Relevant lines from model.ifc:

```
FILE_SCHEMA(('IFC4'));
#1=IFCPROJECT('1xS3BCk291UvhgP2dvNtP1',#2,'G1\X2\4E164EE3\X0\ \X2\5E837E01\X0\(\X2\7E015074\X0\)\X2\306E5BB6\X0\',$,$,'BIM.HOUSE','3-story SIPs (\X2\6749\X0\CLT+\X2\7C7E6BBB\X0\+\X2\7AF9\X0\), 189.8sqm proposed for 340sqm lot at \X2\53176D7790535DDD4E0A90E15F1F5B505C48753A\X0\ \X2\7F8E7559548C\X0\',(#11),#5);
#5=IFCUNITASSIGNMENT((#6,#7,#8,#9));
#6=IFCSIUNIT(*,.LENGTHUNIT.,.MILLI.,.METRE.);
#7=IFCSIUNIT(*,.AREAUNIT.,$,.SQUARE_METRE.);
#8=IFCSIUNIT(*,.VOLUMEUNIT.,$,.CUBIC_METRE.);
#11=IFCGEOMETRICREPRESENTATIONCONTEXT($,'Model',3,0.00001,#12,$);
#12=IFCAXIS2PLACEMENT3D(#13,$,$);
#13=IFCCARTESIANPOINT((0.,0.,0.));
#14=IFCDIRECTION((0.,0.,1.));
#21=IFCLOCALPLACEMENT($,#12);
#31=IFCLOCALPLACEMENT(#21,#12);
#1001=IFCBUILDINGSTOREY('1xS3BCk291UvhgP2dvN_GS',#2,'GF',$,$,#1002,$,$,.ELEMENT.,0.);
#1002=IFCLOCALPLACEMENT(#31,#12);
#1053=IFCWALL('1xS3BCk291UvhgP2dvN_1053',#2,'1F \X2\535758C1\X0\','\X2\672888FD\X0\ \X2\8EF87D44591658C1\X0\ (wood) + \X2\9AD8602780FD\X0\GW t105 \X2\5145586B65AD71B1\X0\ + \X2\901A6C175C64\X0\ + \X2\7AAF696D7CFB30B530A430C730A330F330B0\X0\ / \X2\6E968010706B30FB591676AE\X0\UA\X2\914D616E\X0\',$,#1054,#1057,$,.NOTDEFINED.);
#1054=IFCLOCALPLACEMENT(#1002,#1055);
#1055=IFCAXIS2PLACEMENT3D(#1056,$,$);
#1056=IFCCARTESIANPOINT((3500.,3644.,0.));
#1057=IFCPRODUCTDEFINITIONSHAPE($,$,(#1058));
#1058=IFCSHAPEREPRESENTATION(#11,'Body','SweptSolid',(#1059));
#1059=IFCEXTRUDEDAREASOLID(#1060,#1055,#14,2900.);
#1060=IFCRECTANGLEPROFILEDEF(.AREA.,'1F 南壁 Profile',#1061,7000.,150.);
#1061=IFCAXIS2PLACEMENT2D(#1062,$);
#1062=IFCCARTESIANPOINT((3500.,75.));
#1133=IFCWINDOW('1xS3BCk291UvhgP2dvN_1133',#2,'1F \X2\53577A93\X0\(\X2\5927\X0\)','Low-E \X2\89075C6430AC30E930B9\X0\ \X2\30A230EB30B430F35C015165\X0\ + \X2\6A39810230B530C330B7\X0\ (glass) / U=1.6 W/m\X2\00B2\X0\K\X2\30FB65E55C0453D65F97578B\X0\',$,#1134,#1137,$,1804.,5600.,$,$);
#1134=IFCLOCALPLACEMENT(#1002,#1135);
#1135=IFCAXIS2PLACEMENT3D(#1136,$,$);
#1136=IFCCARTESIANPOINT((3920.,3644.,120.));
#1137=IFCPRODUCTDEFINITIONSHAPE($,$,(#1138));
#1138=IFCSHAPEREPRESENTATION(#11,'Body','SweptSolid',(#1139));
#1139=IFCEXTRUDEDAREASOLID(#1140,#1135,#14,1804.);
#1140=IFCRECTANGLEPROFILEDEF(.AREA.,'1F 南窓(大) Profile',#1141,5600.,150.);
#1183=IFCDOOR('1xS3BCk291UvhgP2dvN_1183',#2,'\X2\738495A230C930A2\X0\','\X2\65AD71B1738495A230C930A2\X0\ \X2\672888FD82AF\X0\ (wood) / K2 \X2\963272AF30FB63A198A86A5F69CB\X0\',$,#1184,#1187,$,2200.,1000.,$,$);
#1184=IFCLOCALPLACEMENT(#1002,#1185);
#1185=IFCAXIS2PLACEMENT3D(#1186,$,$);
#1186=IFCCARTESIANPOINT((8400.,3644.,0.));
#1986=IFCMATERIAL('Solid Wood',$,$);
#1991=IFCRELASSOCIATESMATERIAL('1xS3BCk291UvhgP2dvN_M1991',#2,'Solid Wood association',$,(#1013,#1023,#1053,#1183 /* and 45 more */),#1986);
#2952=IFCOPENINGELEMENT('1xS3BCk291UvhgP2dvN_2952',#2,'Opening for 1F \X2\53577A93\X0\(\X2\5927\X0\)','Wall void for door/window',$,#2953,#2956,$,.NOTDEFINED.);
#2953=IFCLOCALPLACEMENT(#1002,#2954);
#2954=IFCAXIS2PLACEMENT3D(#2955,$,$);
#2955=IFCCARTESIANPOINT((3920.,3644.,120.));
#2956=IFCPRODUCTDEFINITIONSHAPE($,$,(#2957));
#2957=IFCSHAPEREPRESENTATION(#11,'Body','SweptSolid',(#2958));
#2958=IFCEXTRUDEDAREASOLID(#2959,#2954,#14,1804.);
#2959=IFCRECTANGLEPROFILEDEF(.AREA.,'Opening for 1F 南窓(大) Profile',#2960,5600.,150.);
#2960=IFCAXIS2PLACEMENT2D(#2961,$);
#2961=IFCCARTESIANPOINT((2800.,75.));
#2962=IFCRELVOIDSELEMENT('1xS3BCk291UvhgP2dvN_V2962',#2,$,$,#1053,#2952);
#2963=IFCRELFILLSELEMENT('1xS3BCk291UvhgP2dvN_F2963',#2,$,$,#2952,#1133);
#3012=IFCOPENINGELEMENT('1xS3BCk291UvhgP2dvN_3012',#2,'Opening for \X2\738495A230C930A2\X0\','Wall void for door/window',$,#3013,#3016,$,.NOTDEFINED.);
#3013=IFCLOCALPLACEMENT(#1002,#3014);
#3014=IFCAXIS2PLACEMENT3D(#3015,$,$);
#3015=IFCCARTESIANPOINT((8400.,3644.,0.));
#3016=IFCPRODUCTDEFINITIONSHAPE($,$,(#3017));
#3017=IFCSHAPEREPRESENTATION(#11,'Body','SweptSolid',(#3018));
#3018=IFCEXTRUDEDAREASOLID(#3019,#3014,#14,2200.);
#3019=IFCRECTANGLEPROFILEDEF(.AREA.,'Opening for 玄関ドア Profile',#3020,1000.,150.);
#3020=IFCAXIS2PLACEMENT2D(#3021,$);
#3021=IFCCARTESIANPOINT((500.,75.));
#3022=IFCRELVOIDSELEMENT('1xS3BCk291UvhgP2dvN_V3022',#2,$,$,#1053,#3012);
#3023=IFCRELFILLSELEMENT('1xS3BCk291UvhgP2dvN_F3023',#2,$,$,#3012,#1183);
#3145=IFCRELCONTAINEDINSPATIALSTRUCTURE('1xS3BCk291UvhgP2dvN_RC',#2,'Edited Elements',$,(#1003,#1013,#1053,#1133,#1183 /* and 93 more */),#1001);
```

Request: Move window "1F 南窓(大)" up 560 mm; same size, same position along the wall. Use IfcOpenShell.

```python
import numpy as np
import ifcopenshell
import ifcopenshell.api.geometry
import ifcopenshell.util.placement
import ifcopenshell.util.unit

model = ifcopenshell.open("model.ifc")
unit_scale = ifcopenshell.util.unit.calculate_unit_scale(model)

window = model.by_id(1133)
opening = window.FillsVoids[0].RelatingOpeningElement
dz = 0.56 / unit_scale

shift = np.array([0.0, 0.0, dz])
# The window is not placed relative to its opening, so move both.
for product in (opening, window):
    matrix = ifcopenshell.util.placement.get_local_placement(product.ObjectPlacement)
    matrix[:3, 3] += shift
    ifcopenshell.api.geometry.edit_object_placement(model, product=product, matrix=matrix, is_si=False)

print(f"moved by {dz * unit_scale:+.3f} m")

model.write("model_v2.ifc")
```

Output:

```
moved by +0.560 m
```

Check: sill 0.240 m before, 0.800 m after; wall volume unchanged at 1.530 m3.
